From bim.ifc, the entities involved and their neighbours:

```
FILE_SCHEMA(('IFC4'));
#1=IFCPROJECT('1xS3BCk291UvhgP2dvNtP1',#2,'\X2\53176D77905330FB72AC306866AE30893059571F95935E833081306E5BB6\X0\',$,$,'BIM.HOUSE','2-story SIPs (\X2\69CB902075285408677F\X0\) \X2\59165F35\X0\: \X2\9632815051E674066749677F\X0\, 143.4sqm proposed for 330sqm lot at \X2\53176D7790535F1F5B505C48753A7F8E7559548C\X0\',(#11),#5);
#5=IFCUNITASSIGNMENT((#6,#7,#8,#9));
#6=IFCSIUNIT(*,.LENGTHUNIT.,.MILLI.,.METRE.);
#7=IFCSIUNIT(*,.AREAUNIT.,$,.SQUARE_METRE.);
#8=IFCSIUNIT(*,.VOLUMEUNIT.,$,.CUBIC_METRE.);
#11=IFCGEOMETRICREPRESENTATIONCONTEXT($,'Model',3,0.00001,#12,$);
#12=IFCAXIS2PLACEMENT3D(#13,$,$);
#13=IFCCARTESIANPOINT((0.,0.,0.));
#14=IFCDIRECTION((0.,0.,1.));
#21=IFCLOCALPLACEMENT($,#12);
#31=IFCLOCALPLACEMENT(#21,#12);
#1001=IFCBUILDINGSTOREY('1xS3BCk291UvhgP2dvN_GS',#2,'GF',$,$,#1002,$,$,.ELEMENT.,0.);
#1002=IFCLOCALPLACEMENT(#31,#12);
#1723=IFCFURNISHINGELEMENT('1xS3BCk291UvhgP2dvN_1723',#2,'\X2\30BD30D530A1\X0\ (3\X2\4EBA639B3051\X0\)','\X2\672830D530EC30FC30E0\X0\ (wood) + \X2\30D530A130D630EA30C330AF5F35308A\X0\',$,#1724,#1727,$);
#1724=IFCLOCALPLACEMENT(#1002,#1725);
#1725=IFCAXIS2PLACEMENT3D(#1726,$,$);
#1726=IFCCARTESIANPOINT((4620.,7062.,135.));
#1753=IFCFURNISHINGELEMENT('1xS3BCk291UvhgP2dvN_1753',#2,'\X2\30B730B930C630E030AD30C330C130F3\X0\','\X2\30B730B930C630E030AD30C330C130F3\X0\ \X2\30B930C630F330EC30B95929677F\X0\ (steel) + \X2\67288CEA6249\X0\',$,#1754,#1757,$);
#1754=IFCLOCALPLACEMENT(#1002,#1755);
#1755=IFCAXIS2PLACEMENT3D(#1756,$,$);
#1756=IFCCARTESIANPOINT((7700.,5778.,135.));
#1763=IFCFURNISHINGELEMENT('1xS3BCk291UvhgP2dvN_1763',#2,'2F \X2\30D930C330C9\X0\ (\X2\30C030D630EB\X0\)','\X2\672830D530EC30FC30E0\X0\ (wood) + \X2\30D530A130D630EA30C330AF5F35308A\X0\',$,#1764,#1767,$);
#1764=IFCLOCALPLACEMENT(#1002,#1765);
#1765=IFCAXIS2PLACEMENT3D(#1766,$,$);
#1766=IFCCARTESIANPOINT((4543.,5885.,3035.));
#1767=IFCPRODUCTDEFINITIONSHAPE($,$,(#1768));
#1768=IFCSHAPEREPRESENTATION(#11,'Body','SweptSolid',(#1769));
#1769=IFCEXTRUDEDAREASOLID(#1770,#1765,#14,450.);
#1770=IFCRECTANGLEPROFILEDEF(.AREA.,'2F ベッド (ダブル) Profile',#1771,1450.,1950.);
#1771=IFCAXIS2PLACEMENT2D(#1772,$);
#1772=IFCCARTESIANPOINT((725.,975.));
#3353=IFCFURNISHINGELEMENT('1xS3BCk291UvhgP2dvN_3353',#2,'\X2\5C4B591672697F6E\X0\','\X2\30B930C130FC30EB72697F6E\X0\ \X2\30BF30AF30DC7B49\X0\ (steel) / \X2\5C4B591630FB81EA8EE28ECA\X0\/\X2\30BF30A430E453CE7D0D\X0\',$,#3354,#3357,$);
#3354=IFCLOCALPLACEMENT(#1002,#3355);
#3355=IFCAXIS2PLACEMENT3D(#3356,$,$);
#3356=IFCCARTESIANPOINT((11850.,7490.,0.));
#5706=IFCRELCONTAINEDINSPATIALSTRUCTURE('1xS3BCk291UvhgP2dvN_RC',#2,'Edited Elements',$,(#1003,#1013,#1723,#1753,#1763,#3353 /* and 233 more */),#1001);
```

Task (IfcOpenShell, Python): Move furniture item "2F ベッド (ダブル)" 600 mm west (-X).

```python
import ifcopenshell
import ifcopenshell.api.geometry
import ifcopenshell.util.placement
import ifcopenshell.util.unit

model = ifcopenshell.open("bim.ifc")
unit_scale = ifcopenshell.util.unit.calculate_unit_scale(model)

item = model.by_guid("1xS3BCk291UvhgP2dvN_1763")
matrix = ifcopenshell.util.placement.get_local_placement(item.ObjectPlacement)
matrix[0, 3] -= 0.6 / unit_scale
ifcopenshell.api.geometry.edit_object_placement(model, product=item, matrix=matrix, is_si=False)

print(ifcopenshell.util.placement.get_local_placement(item.ObjectPlacement).round(3) + 0.0)

model.write("bim_updated.ifc")
```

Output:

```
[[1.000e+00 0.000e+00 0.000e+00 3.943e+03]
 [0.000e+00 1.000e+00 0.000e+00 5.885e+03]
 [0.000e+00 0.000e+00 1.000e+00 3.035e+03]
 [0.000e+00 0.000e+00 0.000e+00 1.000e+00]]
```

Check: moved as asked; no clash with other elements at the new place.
